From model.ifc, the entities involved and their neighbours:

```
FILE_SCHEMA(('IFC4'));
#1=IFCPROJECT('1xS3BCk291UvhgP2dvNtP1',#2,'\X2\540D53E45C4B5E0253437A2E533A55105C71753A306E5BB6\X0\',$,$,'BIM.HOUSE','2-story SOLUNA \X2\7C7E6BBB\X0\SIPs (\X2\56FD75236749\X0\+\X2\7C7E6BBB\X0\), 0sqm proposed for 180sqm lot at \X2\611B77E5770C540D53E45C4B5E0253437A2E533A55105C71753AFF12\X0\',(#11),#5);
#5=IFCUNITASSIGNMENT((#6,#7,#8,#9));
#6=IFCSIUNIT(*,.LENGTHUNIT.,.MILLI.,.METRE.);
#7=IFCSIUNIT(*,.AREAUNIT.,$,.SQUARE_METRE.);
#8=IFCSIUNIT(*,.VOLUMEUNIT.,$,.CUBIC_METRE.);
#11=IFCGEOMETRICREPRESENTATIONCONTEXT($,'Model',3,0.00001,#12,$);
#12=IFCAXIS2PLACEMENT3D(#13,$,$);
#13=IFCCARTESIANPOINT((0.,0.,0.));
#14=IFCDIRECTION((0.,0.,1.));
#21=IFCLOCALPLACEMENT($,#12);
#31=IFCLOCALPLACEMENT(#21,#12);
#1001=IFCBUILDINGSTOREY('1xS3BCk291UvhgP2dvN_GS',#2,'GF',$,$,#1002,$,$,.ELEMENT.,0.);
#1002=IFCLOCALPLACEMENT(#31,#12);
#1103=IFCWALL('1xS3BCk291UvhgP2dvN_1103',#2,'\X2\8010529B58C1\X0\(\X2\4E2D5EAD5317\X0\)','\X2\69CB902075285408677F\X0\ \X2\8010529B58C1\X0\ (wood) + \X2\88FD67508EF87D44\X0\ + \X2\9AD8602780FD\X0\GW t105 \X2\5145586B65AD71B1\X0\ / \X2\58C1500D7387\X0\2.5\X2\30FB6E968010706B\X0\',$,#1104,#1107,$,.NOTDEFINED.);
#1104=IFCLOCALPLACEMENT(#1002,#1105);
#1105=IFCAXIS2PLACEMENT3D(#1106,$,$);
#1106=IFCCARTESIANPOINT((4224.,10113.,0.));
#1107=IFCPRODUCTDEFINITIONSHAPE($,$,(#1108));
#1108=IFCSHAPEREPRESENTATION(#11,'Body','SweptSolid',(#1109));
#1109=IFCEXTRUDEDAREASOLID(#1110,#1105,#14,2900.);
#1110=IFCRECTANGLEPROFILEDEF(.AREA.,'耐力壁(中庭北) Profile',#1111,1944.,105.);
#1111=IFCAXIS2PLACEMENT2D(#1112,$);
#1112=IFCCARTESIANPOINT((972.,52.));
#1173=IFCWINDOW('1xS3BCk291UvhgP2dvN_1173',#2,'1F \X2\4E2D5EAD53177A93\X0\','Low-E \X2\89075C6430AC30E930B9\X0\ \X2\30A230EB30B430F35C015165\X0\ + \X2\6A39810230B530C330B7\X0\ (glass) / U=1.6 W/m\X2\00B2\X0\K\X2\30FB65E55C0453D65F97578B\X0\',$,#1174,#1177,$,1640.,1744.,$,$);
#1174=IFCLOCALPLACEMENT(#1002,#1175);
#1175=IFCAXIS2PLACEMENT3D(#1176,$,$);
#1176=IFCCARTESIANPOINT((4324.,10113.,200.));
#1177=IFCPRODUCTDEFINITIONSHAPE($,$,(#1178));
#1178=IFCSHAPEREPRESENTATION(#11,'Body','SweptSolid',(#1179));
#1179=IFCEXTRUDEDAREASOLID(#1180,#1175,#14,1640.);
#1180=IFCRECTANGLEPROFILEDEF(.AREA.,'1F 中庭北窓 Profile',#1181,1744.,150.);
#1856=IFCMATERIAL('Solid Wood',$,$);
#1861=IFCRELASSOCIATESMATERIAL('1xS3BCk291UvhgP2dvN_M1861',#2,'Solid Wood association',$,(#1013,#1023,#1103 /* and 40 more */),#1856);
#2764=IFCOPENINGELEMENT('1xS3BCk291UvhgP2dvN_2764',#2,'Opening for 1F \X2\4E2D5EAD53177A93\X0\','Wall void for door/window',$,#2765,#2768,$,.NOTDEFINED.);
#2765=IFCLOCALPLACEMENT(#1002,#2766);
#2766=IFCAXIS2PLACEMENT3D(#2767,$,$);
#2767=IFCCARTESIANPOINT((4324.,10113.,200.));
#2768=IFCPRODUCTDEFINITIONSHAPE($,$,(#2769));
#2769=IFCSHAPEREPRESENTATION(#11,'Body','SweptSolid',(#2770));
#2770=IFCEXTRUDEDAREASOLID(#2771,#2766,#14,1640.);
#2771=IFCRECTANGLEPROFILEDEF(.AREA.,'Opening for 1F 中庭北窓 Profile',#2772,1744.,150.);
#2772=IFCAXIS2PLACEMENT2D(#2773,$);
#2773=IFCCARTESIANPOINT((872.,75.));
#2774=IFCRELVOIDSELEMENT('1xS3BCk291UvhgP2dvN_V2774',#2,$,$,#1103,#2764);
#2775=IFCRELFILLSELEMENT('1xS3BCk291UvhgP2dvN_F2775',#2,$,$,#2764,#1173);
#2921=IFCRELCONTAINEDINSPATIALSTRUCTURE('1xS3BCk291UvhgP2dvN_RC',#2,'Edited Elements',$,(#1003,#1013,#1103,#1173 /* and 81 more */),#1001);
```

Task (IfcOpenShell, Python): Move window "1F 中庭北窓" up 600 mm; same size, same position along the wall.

```python
import numpy as np
import ifcopenshell
import ifcopenshell.api.geometry
import ifcopenshell.util.placement
import ifcopenshell.util.unit

model = ifcopenshell.open("model.ifc")
unit_scale = ifcopenshell.util.unit.calculate_unit_scale(model)

window = model.by_guid("1xS3BCk291UvhgP2dvN_1173")
opening = window.FillsVoids[0].RelatingOpeningElement
dz = 0.6 / unit_scale

shift = np.array([0.0, 0.0, dz])
# The window is not placed relative to its opening, so move both.
for product in (opening, window):
    matrix = ifcopenshell.util.placement.get_local_placement(product.ObjectPlacement)
    matrix[:3, 3] += shift
    ifcopenshell.api.geometry.edit_object_placement(model, product=product, matrix=matrix, is_si=False)

print(f"moved by {dz * unit_scale:+.3f} m")

model.write("model_updated.ifc")
```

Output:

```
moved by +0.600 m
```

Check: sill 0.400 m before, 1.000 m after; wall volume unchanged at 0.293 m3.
